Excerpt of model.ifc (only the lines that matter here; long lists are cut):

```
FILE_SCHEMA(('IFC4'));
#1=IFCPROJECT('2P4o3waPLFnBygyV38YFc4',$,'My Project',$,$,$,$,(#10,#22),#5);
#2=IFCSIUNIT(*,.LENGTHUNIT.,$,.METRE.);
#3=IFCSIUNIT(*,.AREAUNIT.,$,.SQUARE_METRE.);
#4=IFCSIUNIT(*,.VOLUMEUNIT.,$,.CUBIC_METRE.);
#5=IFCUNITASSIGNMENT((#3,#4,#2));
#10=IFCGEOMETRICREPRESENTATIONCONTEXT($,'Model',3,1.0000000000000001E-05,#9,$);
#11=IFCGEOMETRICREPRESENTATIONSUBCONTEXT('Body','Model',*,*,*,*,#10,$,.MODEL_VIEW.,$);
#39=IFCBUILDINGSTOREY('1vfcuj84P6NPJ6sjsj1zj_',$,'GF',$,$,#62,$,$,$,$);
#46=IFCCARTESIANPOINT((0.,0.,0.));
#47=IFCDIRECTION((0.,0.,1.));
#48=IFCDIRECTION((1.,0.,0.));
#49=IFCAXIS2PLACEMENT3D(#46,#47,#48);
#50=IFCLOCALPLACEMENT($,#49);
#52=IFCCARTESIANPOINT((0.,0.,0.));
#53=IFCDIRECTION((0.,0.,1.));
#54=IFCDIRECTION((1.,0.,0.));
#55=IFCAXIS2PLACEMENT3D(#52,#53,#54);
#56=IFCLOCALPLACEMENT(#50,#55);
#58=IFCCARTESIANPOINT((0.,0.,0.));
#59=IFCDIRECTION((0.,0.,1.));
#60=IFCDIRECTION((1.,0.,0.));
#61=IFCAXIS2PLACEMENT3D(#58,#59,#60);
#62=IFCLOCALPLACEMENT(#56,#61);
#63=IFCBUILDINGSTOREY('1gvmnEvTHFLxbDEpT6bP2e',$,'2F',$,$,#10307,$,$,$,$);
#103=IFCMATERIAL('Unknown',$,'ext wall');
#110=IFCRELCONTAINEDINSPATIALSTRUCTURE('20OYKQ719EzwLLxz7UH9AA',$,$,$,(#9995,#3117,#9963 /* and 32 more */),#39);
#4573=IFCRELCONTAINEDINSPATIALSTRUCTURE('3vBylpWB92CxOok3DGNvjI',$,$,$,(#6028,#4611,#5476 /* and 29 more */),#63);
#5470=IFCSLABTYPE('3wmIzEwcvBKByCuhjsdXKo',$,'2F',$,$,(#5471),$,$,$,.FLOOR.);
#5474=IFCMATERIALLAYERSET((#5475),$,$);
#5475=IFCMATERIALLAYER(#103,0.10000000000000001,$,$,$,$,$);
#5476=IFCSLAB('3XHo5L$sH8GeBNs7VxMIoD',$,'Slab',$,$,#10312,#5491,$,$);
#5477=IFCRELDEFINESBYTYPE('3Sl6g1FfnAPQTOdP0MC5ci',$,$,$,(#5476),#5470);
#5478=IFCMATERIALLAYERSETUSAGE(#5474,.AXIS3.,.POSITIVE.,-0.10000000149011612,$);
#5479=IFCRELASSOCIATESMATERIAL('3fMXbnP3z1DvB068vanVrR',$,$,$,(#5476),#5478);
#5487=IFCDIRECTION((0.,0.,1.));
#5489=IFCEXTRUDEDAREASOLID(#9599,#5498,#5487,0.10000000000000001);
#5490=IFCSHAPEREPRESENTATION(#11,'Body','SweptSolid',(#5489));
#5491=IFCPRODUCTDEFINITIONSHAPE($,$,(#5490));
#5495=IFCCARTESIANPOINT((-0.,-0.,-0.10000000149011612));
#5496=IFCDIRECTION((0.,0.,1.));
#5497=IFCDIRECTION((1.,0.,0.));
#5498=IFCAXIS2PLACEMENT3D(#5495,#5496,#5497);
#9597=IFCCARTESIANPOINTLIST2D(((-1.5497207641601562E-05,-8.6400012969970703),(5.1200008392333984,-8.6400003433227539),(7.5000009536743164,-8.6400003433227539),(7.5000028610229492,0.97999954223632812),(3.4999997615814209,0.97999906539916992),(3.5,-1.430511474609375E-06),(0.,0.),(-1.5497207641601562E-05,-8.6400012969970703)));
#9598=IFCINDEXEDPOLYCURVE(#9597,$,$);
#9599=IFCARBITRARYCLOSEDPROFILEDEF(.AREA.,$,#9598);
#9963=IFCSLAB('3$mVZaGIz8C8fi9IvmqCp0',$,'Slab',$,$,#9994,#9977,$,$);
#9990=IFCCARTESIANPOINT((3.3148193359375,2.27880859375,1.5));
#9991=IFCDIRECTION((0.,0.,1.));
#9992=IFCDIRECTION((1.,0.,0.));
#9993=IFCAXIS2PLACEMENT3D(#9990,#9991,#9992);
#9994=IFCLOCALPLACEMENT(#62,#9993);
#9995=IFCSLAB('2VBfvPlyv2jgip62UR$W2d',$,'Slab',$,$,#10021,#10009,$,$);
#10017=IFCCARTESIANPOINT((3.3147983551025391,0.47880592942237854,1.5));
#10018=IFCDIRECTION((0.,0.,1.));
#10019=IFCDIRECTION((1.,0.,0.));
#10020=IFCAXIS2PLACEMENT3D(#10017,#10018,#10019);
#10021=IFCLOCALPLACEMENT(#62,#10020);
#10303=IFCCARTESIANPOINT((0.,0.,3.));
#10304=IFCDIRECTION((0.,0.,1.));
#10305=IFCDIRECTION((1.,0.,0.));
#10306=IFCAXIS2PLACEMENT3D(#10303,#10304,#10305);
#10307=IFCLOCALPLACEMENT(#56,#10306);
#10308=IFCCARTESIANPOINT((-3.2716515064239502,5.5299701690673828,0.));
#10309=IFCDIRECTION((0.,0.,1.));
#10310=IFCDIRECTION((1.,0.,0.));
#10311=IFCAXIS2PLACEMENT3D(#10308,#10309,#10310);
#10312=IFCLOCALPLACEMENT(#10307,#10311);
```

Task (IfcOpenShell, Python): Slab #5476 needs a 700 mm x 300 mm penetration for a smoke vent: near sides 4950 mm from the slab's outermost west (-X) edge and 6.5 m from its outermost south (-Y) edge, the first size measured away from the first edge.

```python
import numpy as np
import ifcopenshell
import ifcopenshell.api.feature
import ifcopenshell.api.geometry
import ifcopenshell.api.root
import ifcopenshell.geom
import ifcopenshell.util.placement
import ifcopenshell.util.representation
import ifcopenshell.util.shape
import ifcopenshell.util.unit

model = ifcopenshell.open("model.ifc")
unit_scale = ifcopenshell.util.unit.calculate_unit_scale(model)
settings = ifcopenshell.geom.settings()


def volume(element):
    """Net volume in cubic metres, openings subtracted."""
    shape = ifcopenshell.geom.create_shape(settings, element)
    return ifcopenshell.util.shape.get_volume(shape.geometry)


slab = model.by_guid("3XHo5L$sH8GeBNs7VxMIoD")
before = volume(slab)

# Extent in the slab's own axes, in metres. The edges named are its -X and -Y sides.
slab_shape = ifcopenshell.geom.create_shape(settings, slab)
vertices = ifcopenshell.util.shape.get_vertices(slab_shape.geometry)
x_min, y_min, bottom = vertices.min(axis=0)
top = vertices[:, 2].max()

opening = ifcopenshell.api.root.create_entity(model, ifc_class="IfcOpeningElement", name="Smoke vent opening", predefined_type="OPENING")
context = ifcopenshell.util.representation.get_context(model, "Model", "Body", "MODEL_VIEW")
width, depth = 0.7, 0.3
outline = [(0.0, 0.0), (width, 0.0), (width, depth), (0.0, depth), (0.0, 0.0)]
# Overshoot both faces by 50 mm so the cut is clean.
shape = ifcopenshell.api.geometry.add_slab_representation(
    model, context=context, depth=top - bottom + 0.1, polyline=outline
)
ifcopenshell.api.geometry.assign_representation(model, product=opening, representation=shape)

matrix = ifcopenshell.util.placement.get_local_placement(slab.ObjectPlacement)
matrix[:, 3] = matrix @ np.append(np.array([x_min + 4.95, y_min + 6.5, bottom - 0.05]) / unit_scale, 1.0)
ifcopenshell.api.geometry.edit_object_placement(model, product=opening, matrix=matrix, is_si=False)
ifcopenshell.api.feature.add_feature(model, feature=opening, element=slab)

after = volume(slab)

print(f"slab volume {before:.3f} -> {after:.3f} m3")

model.write("model_v2.ifc")
```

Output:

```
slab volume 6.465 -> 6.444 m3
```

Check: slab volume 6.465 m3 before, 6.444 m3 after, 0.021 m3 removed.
